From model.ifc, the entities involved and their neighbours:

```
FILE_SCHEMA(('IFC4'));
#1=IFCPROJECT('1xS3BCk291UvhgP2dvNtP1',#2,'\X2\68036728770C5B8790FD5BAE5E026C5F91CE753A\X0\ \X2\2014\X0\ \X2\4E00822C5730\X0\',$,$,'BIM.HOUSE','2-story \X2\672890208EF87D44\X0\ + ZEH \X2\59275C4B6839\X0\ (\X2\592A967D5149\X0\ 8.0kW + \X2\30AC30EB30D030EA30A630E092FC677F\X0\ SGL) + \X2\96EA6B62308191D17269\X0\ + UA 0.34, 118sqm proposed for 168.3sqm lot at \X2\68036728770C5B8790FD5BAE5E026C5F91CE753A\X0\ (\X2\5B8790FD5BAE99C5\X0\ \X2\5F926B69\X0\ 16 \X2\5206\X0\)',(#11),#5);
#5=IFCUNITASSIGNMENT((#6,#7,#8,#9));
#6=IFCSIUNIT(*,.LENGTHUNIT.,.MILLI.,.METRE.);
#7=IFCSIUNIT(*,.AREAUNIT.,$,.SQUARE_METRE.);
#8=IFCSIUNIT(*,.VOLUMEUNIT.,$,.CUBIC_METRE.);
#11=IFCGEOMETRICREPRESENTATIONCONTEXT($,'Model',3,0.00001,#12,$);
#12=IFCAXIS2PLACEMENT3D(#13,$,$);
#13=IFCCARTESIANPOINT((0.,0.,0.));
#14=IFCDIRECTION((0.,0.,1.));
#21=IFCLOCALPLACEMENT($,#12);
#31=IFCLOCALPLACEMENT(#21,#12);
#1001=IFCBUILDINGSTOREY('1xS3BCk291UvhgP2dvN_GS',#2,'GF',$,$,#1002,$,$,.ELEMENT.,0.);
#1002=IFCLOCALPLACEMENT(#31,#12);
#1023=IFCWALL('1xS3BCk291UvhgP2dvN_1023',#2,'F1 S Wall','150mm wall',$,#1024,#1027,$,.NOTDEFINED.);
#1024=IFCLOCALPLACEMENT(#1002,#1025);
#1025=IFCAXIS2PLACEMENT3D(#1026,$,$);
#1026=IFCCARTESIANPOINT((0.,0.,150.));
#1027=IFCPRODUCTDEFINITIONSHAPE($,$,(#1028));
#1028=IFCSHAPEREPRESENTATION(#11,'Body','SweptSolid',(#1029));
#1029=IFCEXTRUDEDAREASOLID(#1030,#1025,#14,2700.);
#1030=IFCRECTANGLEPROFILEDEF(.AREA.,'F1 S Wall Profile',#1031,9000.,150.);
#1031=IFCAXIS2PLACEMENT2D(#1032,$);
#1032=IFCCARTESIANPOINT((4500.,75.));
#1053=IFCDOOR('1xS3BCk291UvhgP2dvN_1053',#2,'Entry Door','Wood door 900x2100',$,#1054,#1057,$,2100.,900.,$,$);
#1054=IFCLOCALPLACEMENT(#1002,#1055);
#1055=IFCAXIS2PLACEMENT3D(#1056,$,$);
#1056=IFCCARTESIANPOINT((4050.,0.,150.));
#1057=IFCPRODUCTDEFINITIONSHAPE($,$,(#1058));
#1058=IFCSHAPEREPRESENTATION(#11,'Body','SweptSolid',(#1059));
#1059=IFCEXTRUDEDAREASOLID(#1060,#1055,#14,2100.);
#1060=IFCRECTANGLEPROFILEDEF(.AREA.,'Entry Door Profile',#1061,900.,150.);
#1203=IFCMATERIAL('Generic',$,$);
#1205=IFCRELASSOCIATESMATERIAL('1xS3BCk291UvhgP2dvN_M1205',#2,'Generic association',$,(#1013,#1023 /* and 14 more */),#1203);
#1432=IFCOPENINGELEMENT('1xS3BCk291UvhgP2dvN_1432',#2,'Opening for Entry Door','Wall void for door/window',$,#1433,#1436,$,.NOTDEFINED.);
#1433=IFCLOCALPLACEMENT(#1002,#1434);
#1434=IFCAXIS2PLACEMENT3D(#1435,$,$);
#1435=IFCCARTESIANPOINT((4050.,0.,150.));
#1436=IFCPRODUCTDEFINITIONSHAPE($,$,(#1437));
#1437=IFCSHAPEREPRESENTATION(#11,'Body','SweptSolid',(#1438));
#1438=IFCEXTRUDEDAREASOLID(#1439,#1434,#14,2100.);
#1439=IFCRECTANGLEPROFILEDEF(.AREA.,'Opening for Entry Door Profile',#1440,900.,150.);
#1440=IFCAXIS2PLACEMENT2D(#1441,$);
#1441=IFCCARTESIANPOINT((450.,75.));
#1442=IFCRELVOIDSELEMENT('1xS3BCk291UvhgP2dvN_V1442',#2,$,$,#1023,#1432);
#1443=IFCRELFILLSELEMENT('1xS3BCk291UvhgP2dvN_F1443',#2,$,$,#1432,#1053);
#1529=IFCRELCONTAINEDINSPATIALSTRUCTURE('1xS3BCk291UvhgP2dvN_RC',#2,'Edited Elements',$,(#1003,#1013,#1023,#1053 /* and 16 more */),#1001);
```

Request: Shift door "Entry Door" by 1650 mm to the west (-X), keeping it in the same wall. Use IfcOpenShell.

```python
import ifcopenshell
import ifcopenshell.api.geometry
import ifcopenshell.util.placement
import ifcopenshell.util.unit

model = ifcopenshell.open("model.ifc")
unit_scale = ifcopenshell.util.unit.calculate_unit_scale(model)

door = model.by_id(1053)
opening = door.FillsVoids[0].RelatingOpeningElement
wall = opening.VoidsElements[0].RelatingBuildingElement

wall_matrix = ifcopenshell.util.placement.get_local_placement(wall.ObjectPlacement)
shift = wall_matrix[:3, 0] * -1.65 / unit_scale
before = ifcopenshell.util.placement.get_local_placement(door.ObjectPlacement)[:3, 3].copy()

# The door is not placed relative to its opening, so move both.
for product in (opening, door):
    matrix = ifcopenshell.util.placement.get_local_placement(product.ObjectPlacement)
    matrix[:3, 3] += shift
    ifcopenshell.api.geometry.edit_object_placement(model, product=product, matrix=matrix, is_si=False)

after = ifcopenshell.util.placement.get_local_placement(door.ObjectPlacement)[:3, 3]
print("door moved by", (after - before).round(3) + 0.0)

model.write("model_rev.ifc")
```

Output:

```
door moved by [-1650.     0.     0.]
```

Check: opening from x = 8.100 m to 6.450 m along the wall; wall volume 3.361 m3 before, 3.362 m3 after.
